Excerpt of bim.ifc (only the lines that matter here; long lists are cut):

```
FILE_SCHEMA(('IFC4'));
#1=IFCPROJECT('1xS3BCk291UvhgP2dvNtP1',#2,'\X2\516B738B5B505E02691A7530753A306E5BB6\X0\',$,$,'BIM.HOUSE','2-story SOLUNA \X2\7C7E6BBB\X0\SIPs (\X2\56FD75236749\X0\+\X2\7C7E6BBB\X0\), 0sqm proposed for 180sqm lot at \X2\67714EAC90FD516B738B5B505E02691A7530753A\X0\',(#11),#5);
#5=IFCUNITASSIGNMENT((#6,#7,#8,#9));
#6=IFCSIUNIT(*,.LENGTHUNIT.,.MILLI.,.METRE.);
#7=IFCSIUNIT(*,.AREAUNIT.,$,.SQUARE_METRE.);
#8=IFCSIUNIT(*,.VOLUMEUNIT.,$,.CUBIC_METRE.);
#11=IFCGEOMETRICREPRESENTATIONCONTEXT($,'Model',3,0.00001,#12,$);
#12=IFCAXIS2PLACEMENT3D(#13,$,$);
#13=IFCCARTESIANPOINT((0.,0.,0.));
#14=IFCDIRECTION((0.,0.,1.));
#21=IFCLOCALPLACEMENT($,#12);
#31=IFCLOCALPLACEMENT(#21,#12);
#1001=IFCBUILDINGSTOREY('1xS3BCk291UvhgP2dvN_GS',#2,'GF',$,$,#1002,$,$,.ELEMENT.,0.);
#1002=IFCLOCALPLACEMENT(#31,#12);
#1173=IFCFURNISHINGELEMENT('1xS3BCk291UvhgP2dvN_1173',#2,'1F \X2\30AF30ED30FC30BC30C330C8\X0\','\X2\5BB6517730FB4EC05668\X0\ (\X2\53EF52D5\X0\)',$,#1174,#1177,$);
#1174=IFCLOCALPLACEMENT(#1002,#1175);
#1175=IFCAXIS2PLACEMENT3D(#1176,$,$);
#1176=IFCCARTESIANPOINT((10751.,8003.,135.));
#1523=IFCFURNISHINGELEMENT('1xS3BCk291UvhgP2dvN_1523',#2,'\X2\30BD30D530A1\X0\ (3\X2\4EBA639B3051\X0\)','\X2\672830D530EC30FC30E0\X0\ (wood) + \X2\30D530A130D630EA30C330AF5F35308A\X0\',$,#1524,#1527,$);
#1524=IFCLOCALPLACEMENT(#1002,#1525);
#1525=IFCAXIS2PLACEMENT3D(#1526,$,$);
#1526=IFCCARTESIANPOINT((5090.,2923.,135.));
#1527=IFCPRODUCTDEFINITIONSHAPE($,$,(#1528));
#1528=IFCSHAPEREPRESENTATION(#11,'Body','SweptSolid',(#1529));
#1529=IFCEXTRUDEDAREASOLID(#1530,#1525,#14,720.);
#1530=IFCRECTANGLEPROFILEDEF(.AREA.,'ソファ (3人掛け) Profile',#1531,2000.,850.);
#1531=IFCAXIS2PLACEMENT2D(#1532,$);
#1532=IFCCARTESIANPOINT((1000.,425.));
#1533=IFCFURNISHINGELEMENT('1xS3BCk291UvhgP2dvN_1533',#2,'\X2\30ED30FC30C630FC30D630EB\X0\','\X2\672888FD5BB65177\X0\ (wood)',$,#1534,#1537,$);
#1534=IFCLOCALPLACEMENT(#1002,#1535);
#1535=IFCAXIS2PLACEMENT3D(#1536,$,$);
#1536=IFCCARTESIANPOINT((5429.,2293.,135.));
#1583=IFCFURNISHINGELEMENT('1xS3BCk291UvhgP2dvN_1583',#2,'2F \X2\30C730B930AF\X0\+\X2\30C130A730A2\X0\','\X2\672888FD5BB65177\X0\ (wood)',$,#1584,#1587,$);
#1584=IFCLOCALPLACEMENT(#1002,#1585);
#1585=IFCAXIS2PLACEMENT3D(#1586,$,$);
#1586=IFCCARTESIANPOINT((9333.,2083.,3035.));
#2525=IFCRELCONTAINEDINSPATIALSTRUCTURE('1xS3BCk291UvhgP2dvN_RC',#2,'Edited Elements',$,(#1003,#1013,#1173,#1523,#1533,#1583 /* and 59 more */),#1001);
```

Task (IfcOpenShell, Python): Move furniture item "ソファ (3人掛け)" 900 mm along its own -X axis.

```python
import ifcopenshell
import ifcopenshell.api.geometry
import ifcopenshell.util.placement
import ifcopenshell.util.unit

model = ifcopenshell.open("bim.ifc")
unit_scale = ifcopenshell.util.unit.calculate_unit_scale(model)

item = model.by_guid("1xS3BCk291UvhgP2dvN_1523")
matrix = ifcopenshell.util.placement.get_local_placement(item.ObjectPlacement)
matrix[:3, 3] -= matrix[:3, 0] * 0.9 / unit_scale
ifcopenshell.api.geometry.edit_object_placement(model, product=item, matrix=matrix, is_si=False)

print(ifcopenshell.util.placement.get_local_placement(item.ObjectPlacement).round(3) + 0.0)

model.write("bim_rev.ifc")
```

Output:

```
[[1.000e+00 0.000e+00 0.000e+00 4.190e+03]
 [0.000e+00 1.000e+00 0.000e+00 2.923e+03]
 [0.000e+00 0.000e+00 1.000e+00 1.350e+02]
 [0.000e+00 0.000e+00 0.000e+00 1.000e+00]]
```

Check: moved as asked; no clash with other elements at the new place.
